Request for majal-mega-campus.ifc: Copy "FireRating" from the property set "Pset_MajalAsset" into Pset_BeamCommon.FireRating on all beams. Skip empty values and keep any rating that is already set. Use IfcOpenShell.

First a look at what the model holds.

```python
import ifcopenshell
import ifcopenshell.util.element

model = ifcopenshell.open("majal-mega-campus.ifc")
print(model.schema)
beams = model.by_type("IfcBeam")
print(len(beams), "beams")
for e in beams[:8]:
    source = ifcopenshell.util.element.get_pset(e, "Pset_MajalAsset", "FireRating")
    target = ifcopenshell.util.element.get_pset(e, "Pset_BeamCommon", "FireRating")
    print(e.id(), repr(source), repr(target), sep=" | ")
```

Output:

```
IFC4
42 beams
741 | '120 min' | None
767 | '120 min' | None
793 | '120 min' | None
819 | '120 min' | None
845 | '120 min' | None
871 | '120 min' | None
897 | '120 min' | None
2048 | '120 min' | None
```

```python
import ifcopenshell
import ifcopenshell.api.pset
import ifcopenshell.util.element

model = ifcopenshell.open("majal-mega-campus.ifc")

count = 0
for e in model.by_type("IfcBeam"):
    value = ifcopenshell.util.element.get_pset(e, "Pset_MajalAsset", "FireRating")
    current = ifcopenshell.util.element.get_pset(e, "Pset_BeamCommon", "FireRating")
    if not value or not value.strip() or current:
        continue
    # add_pset returns the element's existing set when there is one.
    pset = ifcopenshell.api.pset.add_pset(model, product=e, name="Pset_BeamCommon")
    ifcopenshell.api.pset.edit_pset(model, pset=pset, properties={"FireRating": value})
    count += 1

print(count, "beams updated")

model.write("majal-mega-campus_edited.ifc")
```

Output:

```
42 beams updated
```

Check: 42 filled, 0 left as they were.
